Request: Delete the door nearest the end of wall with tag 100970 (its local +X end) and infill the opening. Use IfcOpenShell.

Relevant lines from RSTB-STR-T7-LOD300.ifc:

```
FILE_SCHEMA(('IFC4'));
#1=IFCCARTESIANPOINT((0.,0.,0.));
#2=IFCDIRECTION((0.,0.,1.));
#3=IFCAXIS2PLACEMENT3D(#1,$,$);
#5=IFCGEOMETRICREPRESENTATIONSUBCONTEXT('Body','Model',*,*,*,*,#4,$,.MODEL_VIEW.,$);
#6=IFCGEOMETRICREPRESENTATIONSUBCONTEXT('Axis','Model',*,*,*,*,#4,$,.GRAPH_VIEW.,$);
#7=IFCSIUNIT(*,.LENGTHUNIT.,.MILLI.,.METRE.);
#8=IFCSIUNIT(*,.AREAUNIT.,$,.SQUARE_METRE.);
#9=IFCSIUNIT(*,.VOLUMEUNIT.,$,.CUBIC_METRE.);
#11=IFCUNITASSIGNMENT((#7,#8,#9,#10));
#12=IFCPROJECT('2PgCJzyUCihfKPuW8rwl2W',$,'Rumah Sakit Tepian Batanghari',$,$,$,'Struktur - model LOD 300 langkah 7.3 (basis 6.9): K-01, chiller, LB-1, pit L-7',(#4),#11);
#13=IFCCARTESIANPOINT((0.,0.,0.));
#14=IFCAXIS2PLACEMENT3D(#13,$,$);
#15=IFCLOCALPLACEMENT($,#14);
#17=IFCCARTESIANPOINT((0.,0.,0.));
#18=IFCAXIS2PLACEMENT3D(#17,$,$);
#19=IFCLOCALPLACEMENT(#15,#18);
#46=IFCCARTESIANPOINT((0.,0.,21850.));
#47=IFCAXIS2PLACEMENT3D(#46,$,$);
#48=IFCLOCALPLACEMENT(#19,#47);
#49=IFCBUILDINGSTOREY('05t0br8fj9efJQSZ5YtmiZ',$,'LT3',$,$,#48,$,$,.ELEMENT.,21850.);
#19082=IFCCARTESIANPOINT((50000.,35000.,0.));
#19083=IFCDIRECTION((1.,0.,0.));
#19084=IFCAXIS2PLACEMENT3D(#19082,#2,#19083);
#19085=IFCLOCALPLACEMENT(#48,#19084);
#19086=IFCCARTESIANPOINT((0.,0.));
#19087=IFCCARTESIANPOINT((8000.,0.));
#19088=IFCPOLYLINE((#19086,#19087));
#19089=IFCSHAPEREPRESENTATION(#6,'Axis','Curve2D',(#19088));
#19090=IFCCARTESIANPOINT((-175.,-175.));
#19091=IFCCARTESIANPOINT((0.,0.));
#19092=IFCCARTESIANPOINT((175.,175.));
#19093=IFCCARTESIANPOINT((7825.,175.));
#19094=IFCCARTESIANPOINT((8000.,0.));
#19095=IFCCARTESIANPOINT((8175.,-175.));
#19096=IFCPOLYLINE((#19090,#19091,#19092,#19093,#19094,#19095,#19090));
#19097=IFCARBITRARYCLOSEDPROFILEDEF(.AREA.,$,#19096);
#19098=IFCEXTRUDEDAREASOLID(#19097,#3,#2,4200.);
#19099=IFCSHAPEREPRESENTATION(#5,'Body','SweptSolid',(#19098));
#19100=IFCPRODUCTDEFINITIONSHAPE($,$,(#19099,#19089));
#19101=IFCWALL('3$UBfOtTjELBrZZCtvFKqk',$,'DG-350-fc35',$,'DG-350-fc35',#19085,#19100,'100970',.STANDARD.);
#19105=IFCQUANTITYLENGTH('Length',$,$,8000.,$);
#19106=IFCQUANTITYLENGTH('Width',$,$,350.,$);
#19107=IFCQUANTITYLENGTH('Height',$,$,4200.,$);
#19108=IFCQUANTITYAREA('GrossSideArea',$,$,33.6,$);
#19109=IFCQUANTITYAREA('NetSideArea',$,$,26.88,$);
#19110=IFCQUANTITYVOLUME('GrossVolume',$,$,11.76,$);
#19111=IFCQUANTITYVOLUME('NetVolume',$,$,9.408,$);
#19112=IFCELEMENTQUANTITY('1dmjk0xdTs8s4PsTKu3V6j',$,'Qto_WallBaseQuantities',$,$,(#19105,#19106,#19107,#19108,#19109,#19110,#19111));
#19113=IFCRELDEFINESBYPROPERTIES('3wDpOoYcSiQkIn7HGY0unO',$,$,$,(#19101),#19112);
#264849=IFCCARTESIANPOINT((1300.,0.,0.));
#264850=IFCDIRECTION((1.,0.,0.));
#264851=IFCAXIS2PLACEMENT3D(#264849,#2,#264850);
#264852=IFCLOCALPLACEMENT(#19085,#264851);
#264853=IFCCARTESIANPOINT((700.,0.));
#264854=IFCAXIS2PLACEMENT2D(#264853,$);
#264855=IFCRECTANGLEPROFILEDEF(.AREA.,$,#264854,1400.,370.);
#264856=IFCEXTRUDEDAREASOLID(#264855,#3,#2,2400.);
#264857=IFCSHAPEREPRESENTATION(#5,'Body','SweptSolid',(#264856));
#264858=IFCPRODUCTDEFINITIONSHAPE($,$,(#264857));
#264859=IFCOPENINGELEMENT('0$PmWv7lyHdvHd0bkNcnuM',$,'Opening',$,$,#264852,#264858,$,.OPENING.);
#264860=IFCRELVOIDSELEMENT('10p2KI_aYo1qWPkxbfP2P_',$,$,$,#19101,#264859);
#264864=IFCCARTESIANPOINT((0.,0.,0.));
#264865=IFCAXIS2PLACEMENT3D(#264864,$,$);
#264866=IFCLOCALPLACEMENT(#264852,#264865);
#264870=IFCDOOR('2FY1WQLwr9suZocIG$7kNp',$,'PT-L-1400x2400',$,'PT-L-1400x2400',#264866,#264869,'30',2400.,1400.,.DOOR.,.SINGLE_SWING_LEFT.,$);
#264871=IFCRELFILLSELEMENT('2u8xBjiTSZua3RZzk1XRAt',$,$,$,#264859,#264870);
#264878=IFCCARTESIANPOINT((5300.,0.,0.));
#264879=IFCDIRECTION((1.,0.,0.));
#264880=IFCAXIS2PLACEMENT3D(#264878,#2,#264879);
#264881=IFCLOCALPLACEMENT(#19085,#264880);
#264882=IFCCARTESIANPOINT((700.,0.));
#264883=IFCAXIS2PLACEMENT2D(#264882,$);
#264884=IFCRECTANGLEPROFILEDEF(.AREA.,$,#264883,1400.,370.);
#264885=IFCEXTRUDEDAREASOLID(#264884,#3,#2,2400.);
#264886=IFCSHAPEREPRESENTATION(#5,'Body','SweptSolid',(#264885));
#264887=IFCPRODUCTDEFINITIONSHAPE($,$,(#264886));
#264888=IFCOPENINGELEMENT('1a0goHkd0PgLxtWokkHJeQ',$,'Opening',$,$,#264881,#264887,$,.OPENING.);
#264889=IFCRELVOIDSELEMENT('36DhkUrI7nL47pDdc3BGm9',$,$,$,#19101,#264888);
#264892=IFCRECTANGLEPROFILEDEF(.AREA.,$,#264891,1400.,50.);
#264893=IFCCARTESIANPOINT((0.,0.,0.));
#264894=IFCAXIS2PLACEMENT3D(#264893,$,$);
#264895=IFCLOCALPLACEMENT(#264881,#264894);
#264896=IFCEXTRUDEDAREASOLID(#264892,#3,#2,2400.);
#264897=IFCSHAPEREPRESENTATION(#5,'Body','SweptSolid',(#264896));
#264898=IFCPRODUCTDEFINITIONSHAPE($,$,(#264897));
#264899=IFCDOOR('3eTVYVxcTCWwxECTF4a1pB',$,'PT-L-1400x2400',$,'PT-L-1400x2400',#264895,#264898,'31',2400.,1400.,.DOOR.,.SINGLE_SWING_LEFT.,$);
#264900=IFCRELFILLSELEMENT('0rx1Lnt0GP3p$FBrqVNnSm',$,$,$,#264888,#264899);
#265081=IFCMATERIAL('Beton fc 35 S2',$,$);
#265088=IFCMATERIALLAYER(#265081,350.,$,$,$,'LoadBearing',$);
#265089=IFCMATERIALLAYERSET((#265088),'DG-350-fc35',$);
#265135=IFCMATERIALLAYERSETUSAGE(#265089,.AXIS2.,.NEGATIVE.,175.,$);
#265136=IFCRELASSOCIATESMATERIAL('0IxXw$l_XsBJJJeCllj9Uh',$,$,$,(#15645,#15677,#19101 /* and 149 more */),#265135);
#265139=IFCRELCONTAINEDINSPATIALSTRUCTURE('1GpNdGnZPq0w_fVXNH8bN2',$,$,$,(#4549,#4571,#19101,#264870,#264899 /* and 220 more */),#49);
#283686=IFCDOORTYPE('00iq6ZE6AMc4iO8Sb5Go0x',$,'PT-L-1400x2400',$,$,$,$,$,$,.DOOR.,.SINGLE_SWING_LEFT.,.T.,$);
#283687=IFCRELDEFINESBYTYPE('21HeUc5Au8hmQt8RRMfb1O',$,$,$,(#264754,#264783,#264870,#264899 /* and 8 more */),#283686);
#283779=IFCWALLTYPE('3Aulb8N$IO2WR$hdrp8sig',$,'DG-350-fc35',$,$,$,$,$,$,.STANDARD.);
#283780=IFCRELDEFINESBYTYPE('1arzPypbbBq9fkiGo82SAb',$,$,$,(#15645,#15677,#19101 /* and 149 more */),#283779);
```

```python
import ifcopenshell
import ifcopenshell.api.feature
import ifcopenshell.api.pset
import ifcopenshell.api.root
import ifcopenshell.geom
import ifcopenshell.util.element
import ifcopenshell.util.shape
import ifcopenshell.util.unit

model = ifcopenshell.open("RSTB-STR-T7-LOD300.ifc")
area_scale = ifcopenshell.util.unit.calculate_unit_scale(model, "AREAUNIT")
volume_scale = ifcopenshell.util.unit.calculate_unit_scale(model, "VOLUMEUNIT")
settings = ifcopenshell.geom.settings()


def volume(element):
    """Net volume in cubic metres, openings subtracted."""
    shape = ifcopenshell.geom.create_shape(settings, element)
    return ifcopenshell.util.shape.get_volume(shape.geometry)


door = model.by_guid("3eTVYVxcTCWwxECTF4a1pB")
opening = door.FillsVoids[0].RelatingOpeningElement
wall = opening.VoidsElements[0].RelatingBuildingElement
before = volume(wall)

ifcopenshell.api.root.remove_product(model, product=door)
ifcopenshell.api.feature.remove_feature(model, feature=opening)

after = volume(wall)
thickness = 0.35  # wall thickness in metres

# Update the wall's stored quantities.
qto = model.by_id(ifcopenshell.util.element.get_pset(wall, "Qto_WallBaseQuantities", should_inherit=False)["id"])
ifcopenshell.api.pset.edit_qto(model, qto=qto, properties={
    "NetSideArea": after / thickness / area_scale,
    "NetVolume": after / volume_scale,
})

print(f"wall volume {before:.3f} -> {after:.3f} m3")

model.write("RSTB-STR-T7-LOD300_edited.ifc")
```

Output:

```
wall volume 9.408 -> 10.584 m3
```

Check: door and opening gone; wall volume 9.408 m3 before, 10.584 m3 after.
